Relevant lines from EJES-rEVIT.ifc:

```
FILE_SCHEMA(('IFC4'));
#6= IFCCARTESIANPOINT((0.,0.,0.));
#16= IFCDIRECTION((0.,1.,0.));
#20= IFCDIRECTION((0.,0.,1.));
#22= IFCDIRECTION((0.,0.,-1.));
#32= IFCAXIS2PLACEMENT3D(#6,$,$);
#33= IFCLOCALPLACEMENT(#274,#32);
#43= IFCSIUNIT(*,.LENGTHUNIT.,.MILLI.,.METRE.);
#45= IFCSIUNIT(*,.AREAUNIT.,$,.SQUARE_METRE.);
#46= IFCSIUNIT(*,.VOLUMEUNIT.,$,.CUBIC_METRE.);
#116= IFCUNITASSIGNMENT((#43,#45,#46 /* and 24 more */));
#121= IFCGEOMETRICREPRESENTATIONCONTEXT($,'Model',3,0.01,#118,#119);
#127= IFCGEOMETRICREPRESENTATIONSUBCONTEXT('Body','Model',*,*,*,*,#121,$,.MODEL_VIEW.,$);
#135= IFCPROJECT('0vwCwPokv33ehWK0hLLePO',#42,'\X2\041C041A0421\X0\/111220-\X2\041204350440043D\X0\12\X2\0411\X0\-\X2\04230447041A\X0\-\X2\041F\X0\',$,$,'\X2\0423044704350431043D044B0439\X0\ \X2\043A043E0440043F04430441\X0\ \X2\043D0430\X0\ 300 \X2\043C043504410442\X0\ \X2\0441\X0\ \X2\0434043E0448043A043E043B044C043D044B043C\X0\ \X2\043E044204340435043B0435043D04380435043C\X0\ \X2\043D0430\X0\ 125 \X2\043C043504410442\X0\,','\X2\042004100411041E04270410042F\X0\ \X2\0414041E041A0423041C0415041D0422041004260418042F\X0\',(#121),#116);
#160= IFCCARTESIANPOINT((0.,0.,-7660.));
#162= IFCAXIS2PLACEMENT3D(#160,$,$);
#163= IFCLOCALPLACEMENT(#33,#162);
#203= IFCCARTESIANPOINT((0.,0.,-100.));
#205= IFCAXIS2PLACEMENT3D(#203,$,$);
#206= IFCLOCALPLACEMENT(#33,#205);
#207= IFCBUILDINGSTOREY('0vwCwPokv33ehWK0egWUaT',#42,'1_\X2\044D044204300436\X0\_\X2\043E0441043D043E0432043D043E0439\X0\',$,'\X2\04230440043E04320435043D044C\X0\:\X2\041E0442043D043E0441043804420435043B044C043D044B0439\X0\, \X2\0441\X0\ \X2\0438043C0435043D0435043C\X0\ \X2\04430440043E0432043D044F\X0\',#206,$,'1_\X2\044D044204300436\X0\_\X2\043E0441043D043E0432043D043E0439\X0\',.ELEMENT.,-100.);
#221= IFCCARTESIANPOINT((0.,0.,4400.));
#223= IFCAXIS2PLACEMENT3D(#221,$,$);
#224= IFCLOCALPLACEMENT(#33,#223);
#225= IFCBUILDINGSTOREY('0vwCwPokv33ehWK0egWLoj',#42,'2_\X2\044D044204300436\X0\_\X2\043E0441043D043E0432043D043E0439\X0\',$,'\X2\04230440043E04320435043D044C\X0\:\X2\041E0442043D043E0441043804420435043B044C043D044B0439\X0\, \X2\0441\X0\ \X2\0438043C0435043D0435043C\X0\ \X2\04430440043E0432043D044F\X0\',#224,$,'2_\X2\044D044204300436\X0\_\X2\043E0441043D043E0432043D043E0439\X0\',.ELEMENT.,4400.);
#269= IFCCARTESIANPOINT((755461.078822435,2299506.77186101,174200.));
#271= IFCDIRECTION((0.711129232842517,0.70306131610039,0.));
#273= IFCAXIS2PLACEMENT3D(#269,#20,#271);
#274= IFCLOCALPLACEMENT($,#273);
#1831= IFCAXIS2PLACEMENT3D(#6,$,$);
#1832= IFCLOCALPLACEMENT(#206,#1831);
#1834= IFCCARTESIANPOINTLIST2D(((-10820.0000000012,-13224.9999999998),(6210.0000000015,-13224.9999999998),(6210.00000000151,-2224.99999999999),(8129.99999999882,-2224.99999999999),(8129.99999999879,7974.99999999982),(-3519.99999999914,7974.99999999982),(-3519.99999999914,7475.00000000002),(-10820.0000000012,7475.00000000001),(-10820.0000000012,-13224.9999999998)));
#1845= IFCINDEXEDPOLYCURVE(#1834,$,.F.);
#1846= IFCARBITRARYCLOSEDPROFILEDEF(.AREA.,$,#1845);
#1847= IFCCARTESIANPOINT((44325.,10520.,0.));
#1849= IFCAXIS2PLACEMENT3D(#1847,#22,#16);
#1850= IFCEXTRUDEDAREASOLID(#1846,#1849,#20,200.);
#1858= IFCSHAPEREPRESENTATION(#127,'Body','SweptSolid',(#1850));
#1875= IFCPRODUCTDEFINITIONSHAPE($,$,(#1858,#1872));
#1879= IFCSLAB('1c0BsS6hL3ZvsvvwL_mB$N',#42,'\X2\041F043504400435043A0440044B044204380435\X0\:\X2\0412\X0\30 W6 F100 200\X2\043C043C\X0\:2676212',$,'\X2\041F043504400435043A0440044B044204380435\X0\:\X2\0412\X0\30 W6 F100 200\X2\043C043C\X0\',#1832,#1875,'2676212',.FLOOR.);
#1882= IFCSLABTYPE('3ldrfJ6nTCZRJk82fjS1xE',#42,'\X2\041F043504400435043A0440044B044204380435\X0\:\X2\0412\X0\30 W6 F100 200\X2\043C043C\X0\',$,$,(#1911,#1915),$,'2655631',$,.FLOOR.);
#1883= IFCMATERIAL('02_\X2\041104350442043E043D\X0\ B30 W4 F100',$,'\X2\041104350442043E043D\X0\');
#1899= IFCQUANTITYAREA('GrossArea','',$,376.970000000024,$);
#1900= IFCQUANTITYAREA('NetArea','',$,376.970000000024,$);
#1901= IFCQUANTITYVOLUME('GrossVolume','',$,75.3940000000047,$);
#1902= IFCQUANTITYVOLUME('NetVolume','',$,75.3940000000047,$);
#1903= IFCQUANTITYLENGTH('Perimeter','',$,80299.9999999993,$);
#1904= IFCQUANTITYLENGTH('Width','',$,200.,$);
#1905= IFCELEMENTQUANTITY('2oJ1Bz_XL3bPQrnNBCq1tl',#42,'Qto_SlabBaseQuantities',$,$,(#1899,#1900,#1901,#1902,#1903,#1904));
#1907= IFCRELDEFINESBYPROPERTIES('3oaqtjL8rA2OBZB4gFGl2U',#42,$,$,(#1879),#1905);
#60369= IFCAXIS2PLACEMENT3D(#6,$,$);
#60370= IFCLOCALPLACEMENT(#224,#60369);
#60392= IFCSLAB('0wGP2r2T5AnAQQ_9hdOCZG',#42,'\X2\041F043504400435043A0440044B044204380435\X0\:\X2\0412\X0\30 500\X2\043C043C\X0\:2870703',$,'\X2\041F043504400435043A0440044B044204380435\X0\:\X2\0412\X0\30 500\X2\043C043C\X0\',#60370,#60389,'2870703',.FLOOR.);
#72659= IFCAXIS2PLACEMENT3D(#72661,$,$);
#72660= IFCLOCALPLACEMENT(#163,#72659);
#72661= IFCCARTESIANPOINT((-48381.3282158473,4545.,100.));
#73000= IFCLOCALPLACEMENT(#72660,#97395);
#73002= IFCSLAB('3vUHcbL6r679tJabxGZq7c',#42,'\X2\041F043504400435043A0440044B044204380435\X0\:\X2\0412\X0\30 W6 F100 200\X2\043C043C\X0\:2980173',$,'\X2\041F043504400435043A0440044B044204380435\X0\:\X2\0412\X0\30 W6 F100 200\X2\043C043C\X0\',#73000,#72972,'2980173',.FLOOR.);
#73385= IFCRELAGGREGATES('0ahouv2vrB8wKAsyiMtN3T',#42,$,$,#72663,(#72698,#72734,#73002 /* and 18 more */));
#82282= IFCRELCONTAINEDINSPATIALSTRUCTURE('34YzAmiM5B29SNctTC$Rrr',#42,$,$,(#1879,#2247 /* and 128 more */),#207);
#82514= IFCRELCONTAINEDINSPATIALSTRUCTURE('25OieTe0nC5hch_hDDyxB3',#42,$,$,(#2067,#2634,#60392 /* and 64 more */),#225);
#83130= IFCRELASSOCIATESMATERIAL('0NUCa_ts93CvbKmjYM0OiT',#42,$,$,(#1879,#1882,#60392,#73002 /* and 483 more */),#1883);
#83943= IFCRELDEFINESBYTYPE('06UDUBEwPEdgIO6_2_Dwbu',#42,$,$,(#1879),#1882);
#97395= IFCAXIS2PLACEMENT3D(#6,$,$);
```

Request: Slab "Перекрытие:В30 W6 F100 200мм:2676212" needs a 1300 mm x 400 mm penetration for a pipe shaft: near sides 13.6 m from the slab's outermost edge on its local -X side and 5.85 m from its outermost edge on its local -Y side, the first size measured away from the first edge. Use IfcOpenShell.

```python
import numpy as np
import ifcopenshell
import ifcopenshell.api.feature
import ifcopenshell.api.geometry
import ifcopenshell.api.pset
import ifcopenshell.api.root
import ifcopenshell.geom
import ifcopenshell.util.element
import ifcopenshell.util.placement
import ifcopenshell.util.representation
import ifcopenshell.util.shape
import ifcopenshell.util.unit

model = ifcopenshell.open("EJES-rEVIT.ifc")
unit_scale = ifcopenshell.util.unit.calculate_unit_scale(model)
area_scale = ifcopenshell.util.unit.calculate_unit_scale(model, "AREAUNIT")
volume_scale = ifcopenshell.util.unit.calculate_unit_scale(model, "VOLUMEUNIT")
settings = ifcopenshell.geom.settings()


def volume(element):
    """Net volume in cubic metres, openings subtracted."""
    shape = ifcopenshell.geom.create_shape(settings, element)
    return ifcopenshell.util.shape.get_volume(shape.geometry)


slab = model.by_guid("1c0BsS6hL3ZvsvvwL_mB$N")
before = volume(slab)

# Extent in the slab's own axes, in metres. The edges named are its -X and -Y sides.
slab_shape = ifcopenshell.geom.create_shape(settings, slab)
vertices = ifcopenshell.util.shape.get_vertices(slab_shape.geometry)
x_min, y_min, bottom = vertices.min(axis=0)
top = vertices[:, 2].max()

opening = ifcopenshell.api.root.create_entity(model, ifc_class="IfcOpeningElement", name="Pipe shaft opening", predefined_type="OPENING")
context = ifcopenshell.util.representation.get_context(model, "Model", "Body", "MODEL_VIEW")
width, depth = 1.3, 0.4
outline = [(0.0, 0.0), (width, 0.0), (width, depth), (0.0, depth), (0.0, 0.0)]
# Overshoot both faces by 50 mm so the cut is clean.
shape = ifcopenshell.api.geometry.add_slab_representation(
    model, context=context, depth=top - bottom + 0.1, polyline=outline
)
ifcopenshell.api.geometry.assign_representation(model, product=opening, representation=shape)

matrix = ifcopenshell.util.placement.get_local_placement(slab.ObjectPlacement)
matrix[:, 3] = matrix @ np.append(np.array([x_min + 13.6, y_min + 5.85, bottom - 0.05]) / unit_scale, 1.0)
ifcopenshell.api.geometry.edit_object_placement(model, product=opening, matrix=matrix, is_si=False)
ifcopenshell.api.feature.add_feature(model, feature=opening, element=slab)

after = volume(slab)

# Update the slab's stored quantities.
qto = model.by_id(ifcopenshell.util.element.get_pset(slab, "Qto_SlabBaseQuantities", should_inherit=False)["id"])
ifcopenshell.api.pset.edit_qto(model, qto=qto, properties={
    "NetArea": after / (top - bottom) / area_scale,
    "NetVolume": after / volume_scale,
})

print(f"slab volume {before:.3f} -> {after:.3f} m3")

model.write("EJES-rEVIT_v2.ifc")
```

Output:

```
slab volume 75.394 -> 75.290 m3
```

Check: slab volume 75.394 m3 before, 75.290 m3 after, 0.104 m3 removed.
